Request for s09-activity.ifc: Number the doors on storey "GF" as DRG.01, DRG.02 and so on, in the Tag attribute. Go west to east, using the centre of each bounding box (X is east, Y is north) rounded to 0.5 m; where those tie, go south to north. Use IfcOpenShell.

First a look at what the model holds.

```python
import ifcopenshell
import ifcopenshell.util.element
import ifcopenshell.util.placement

model = ifcopenshell.open("s09-activity.ifc")
print(model.schema)
storey = next(s for s in model.by_type("IfcBuildingStorey") if s.Name == "GF")
doors = [e for e in ifcopenshell.util.element.get_decomposition(storey) if e.is_a("IfcDoor")]
for e in sorted(doors, key=lambda e: e.id()):
    origin = ifcopenshell.util.placement.get_local_placement(e.ObjectPlacement)[:3, 3]
    print(e.id(), e.Tag, e.Name, origin.round(2) + 0.0, sep=" | ")
```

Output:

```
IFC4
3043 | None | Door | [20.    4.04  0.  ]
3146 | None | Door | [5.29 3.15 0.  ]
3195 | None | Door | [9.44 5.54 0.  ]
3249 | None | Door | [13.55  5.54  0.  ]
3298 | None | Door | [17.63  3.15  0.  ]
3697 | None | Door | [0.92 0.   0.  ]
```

```python
import ifcopenshell
import ifcopenshell.geom
import ifcopenshell.util.element
import ifcopenshell.util.shape

model = ifcopenshell.open("s09-activity.ifc")
settings = ifcopenshell.geom.settings()
settings.set("use-world-coords", True)


def centre(element):
    shape = ifcopenshell.geom.create_shape(settings, element)
    return ifcopenshell.util.shape.get_bbox_centroid(shape.geometry)


storey = next(s for s in model.by_type("IfcBuildingStorey") if s.Name == "GF")
doors = [e for e in ifcopenshell.util.element.get_decomposition(storey) if e.is_a("IfcDoor")]

# Insertion points can sit at a corner or the storey origin, so sort by the geometry (in metres).
centres = {e: centre(e) for e in doors}
doors.sort(key=lambda e: (round(centres[e][0] / 0.5), centres[e][1]))

for i, e in enumerate(doors, start=1):
    number = f"DRG.{i:02d}"
    e.Tag = number
    print(e.id(), number)

model.write("s09-activity_updated.ifc")
```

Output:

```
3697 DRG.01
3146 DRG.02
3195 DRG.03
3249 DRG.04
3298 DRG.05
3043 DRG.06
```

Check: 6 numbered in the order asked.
